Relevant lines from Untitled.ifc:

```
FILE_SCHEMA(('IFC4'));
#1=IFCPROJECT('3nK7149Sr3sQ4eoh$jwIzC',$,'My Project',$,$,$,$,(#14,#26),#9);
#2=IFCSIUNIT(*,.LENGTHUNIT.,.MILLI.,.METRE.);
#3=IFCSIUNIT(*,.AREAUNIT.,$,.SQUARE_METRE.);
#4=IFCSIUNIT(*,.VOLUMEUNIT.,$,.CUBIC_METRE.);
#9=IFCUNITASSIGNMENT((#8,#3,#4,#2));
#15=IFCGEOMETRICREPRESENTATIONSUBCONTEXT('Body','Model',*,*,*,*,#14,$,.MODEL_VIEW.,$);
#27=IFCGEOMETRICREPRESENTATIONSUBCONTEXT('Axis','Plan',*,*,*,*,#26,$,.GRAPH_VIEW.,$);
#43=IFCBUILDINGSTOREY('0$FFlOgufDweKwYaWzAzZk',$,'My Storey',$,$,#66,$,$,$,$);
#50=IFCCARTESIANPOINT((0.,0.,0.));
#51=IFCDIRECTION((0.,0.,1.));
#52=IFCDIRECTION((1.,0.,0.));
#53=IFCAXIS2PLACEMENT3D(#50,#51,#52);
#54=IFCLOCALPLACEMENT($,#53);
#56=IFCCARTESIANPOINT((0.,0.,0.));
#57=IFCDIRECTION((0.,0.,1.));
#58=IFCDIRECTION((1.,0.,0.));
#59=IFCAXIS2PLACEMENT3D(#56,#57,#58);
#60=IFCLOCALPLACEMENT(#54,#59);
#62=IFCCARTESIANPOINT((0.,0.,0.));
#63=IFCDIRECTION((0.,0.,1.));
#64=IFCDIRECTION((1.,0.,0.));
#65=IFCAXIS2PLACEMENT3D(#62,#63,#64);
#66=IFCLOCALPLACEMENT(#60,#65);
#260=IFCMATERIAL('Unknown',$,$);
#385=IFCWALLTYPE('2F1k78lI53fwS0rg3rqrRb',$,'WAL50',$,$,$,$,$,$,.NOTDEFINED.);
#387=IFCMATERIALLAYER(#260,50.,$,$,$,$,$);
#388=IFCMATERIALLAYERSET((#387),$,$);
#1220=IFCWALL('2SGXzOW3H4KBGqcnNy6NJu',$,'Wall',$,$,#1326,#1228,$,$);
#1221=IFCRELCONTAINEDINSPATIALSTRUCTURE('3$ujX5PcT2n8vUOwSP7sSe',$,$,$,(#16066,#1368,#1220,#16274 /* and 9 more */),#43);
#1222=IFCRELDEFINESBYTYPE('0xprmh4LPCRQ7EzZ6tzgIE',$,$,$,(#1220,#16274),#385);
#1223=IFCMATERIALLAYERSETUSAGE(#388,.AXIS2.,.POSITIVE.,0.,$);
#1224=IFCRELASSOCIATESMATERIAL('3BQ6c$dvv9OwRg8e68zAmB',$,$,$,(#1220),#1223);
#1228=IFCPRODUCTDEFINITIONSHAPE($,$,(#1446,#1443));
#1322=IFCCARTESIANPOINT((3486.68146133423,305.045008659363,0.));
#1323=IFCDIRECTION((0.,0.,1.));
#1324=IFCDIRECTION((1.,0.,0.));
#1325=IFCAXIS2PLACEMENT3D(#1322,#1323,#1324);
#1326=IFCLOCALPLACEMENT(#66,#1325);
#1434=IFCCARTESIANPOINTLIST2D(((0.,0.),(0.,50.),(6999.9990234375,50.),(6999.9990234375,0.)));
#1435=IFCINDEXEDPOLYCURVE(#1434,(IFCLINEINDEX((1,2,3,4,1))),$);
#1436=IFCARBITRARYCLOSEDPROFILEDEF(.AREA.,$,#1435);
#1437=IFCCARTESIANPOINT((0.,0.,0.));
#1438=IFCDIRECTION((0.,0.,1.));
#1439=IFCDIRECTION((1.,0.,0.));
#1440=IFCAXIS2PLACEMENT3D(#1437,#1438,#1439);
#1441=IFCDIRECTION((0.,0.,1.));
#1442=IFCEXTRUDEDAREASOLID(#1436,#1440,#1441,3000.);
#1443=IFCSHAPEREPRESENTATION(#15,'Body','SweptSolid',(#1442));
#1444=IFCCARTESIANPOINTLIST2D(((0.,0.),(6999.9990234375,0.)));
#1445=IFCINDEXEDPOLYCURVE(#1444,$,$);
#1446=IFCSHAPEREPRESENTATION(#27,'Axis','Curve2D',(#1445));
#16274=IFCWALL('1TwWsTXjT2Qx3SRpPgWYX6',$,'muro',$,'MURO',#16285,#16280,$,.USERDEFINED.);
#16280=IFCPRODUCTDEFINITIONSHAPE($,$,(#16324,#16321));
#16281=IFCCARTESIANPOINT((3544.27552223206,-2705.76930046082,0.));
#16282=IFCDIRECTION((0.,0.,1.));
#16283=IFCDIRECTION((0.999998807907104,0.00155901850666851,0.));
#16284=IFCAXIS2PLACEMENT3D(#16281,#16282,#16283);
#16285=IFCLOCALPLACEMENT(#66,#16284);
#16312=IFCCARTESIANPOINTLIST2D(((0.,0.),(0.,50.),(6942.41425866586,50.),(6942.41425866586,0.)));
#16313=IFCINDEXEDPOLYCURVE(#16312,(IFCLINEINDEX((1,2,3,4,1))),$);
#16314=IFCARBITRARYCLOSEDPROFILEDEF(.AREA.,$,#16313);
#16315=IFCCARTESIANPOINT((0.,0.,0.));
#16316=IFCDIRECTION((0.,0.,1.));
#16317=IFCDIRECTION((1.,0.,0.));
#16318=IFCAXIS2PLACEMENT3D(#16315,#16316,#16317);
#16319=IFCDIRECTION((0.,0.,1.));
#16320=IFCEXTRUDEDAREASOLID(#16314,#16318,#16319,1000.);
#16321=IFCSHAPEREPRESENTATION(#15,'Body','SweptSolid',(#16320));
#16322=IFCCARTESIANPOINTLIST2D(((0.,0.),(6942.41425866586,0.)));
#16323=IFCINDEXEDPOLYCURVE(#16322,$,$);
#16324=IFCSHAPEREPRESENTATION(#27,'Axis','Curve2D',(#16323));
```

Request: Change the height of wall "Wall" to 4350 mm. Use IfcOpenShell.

```python
import ifcopenshell
import ifcopenshell.geom
import ifcopenshell.util.representation
import ifcopenshell.util.shape
import ifcopenshell.util.unit

model = ifcopenshell.open("Untitled.ifc")
unit_scale = ifcopenshell.util.unit.calculate_unit_scale(model)
settings = ifcopenshell.geom.settings()


def volume(element):
    """Net volume in cubic metres, openings subtracted."""
    shape = ifcopenshell.geom.create_shape(settings, element)
    return ifcopenshell.util.shape.get_volume(shape.geometry)


wall = model.by_guid("2SGXzOW3H4KBGqcnNy6NJu")
before = volume(wall)

body = ifcopenshell.util.representation.get_representation(wall, "Model", "Body")
solid = body.Items[0]
old_height = solid.Depth
solid.Depth = 4.35 / unit_scale
after = volume(wall)

print(f"height {old_height:g} -> {solid.Depth:g}, volume {before:.3f} -> {after:.3f} m3")

model.write("Untitled_edited.ifc")
```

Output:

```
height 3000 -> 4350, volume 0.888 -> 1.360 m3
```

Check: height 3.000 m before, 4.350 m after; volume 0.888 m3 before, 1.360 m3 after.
